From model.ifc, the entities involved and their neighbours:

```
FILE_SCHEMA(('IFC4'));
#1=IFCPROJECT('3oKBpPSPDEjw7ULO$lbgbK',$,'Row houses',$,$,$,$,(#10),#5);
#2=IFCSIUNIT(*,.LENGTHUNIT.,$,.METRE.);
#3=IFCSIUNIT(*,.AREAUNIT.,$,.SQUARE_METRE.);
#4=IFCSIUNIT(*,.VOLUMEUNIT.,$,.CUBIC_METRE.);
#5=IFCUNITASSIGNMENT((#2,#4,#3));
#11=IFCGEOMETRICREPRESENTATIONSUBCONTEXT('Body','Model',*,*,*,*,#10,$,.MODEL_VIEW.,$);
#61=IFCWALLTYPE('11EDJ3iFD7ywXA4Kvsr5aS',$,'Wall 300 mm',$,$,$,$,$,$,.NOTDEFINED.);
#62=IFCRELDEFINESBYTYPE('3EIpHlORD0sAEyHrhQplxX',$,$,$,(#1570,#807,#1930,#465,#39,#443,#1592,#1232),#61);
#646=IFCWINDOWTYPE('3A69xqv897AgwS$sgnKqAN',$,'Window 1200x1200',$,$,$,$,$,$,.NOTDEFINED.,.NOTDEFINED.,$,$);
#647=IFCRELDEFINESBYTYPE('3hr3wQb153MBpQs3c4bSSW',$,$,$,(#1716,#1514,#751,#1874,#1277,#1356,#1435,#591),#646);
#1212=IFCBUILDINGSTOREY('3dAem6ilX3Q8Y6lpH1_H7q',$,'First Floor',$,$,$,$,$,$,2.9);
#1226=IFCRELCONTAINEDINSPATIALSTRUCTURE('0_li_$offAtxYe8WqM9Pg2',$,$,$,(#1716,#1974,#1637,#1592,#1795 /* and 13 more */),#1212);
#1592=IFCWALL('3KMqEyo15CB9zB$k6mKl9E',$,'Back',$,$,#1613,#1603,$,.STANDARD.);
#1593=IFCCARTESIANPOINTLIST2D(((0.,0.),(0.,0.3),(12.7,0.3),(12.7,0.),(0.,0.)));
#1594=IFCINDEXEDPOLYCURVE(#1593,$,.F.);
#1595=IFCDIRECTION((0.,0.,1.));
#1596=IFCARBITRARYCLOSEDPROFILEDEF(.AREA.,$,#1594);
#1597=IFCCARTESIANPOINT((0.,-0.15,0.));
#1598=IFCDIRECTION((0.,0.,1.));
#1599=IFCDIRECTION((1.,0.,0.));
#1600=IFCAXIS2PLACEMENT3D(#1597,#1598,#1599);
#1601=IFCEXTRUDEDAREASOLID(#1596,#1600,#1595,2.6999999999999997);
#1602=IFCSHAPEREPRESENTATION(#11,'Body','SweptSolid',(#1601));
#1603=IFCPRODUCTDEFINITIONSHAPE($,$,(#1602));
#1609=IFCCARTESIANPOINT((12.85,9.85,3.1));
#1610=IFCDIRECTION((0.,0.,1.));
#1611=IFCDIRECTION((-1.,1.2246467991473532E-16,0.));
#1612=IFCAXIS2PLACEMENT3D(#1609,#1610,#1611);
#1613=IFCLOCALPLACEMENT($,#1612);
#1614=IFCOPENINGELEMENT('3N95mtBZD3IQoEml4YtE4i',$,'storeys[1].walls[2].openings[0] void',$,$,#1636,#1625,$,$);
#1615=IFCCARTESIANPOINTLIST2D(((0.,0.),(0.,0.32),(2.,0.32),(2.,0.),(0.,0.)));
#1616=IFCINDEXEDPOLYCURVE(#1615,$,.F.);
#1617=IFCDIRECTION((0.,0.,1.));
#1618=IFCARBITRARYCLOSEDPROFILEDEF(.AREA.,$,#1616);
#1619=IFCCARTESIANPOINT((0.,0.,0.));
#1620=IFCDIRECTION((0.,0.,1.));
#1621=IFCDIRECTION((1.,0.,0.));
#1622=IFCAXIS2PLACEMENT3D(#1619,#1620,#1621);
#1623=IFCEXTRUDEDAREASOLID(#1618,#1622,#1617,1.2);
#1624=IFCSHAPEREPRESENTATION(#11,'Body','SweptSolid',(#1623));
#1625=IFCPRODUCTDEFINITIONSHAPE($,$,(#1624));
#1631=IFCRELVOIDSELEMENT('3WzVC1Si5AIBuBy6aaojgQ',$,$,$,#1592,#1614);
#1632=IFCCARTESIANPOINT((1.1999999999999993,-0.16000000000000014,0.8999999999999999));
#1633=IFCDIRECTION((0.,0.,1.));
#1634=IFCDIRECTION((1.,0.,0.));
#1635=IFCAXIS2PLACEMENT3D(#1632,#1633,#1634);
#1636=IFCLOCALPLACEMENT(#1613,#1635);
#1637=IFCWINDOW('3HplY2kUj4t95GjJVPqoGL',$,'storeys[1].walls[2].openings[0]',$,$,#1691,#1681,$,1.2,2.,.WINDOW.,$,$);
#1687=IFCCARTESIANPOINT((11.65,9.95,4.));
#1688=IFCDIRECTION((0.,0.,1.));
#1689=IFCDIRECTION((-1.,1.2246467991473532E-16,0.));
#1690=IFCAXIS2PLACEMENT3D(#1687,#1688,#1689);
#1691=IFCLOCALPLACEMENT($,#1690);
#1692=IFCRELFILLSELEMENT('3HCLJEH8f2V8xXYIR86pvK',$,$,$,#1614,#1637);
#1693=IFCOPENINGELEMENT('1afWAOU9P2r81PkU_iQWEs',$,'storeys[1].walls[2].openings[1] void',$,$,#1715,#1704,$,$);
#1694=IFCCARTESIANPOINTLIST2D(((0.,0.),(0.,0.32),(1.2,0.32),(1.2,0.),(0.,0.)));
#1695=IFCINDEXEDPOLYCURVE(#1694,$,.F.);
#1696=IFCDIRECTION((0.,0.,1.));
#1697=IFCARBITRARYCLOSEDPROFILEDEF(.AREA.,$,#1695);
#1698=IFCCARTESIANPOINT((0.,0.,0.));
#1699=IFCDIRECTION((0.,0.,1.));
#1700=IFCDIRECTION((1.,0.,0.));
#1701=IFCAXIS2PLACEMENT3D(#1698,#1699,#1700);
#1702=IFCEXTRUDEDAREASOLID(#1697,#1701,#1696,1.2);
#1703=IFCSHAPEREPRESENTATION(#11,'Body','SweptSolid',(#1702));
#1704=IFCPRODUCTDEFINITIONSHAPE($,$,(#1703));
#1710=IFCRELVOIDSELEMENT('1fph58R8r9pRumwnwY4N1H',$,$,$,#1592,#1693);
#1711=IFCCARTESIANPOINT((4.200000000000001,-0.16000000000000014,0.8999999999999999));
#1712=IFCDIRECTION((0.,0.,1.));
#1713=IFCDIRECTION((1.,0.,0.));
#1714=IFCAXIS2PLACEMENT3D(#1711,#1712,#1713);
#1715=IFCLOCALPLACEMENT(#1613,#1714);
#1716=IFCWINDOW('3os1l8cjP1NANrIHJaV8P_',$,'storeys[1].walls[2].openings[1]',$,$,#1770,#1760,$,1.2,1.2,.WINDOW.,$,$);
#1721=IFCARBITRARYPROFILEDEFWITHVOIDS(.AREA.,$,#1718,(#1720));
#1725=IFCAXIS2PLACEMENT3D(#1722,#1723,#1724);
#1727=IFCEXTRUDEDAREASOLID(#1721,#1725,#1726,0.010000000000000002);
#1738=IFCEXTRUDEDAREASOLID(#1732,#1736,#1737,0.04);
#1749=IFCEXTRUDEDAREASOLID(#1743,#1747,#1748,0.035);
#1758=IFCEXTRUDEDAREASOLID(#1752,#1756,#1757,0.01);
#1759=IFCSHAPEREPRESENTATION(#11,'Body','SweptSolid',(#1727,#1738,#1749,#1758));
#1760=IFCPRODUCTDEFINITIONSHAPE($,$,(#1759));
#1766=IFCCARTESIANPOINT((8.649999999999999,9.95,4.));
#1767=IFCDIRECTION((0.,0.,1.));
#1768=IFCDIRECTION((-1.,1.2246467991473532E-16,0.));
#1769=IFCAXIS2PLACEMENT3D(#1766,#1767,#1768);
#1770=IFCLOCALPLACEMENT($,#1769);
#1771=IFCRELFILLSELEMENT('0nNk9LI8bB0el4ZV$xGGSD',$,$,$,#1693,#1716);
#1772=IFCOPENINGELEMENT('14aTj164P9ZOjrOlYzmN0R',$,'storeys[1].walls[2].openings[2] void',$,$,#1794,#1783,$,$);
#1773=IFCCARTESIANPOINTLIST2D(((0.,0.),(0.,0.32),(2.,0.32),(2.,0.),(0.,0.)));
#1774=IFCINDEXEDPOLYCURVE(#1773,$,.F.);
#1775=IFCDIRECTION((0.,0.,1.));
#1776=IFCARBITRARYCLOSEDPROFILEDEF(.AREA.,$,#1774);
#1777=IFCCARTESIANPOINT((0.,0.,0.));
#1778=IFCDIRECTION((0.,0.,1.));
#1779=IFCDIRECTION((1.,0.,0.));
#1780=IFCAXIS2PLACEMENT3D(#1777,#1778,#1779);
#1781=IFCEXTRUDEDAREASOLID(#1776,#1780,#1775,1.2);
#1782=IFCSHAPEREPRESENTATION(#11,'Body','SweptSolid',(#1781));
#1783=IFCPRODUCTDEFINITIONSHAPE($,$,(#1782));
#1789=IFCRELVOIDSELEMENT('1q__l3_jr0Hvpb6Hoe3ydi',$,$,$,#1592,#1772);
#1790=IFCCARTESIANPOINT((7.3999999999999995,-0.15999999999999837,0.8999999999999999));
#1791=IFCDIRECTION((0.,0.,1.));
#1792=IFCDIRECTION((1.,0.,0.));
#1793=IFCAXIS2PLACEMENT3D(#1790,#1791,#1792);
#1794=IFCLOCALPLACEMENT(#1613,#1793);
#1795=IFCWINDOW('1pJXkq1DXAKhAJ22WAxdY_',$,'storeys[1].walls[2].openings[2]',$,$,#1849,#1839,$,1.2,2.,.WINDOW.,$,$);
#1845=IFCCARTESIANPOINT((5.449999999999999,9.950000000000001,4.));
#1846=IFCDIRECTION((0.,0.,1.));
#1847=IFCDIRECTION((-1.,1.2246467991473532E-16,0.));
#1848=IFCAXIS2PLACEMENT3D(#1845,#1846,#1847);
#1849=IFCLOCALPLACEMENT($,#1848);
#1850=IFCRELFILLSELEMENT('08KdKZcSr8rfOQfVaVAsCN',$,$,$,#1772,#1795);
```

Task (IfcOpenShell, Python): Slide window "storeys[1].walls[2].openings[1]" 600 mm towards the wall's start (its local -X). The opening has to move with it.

```python
import ifcopenshell
import ifcopenshell.api.geometry
import ifcopenshell.util.placement
import ifcopenshell.util.unit

model = ifcopenshell.open("model.ifc")
unit_scale = ifcopenshell.util.unit.calculate_unit_scale(model)

window = model.by_id(1716)
opening = window.FillsVoids[0].RelatingOpeningElement
wall = opening.VoidsElements[0].RelatingBuildingElement

wall_matrix = ifcopenshell.util.placement.get_local_placement(wall.ObjectPlacement)
shift = wall_matrix[:3, 0] * -0.6 / unit_scale
before = ifcopenshell.util.placement.get_local_placement(window.ObjectPlacement)[:3, 3].copy()

# The window is not placed relative to its opening, so move both.
for product in (opening, window):
    matrix = ifcopenshell.util.placement.get_local_placement(product.ObjectPlacement)
    matrix[:3, 3] += shift
    ifcopenshell.api.geometry.edit_object_placement(model, product=product, matrix=matrix, is_si=False)

after = ifcopenshell.util.placement.get_local_placement(window.ObjectPlacement)[:3, 3]
print("window moved by", (after - before).round(3) + 0.0)

model.write("model_updated.ifc")
```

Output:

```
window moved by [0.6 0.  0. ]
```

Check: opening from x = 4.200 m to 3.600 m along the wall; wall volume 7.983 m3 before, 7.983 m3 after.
